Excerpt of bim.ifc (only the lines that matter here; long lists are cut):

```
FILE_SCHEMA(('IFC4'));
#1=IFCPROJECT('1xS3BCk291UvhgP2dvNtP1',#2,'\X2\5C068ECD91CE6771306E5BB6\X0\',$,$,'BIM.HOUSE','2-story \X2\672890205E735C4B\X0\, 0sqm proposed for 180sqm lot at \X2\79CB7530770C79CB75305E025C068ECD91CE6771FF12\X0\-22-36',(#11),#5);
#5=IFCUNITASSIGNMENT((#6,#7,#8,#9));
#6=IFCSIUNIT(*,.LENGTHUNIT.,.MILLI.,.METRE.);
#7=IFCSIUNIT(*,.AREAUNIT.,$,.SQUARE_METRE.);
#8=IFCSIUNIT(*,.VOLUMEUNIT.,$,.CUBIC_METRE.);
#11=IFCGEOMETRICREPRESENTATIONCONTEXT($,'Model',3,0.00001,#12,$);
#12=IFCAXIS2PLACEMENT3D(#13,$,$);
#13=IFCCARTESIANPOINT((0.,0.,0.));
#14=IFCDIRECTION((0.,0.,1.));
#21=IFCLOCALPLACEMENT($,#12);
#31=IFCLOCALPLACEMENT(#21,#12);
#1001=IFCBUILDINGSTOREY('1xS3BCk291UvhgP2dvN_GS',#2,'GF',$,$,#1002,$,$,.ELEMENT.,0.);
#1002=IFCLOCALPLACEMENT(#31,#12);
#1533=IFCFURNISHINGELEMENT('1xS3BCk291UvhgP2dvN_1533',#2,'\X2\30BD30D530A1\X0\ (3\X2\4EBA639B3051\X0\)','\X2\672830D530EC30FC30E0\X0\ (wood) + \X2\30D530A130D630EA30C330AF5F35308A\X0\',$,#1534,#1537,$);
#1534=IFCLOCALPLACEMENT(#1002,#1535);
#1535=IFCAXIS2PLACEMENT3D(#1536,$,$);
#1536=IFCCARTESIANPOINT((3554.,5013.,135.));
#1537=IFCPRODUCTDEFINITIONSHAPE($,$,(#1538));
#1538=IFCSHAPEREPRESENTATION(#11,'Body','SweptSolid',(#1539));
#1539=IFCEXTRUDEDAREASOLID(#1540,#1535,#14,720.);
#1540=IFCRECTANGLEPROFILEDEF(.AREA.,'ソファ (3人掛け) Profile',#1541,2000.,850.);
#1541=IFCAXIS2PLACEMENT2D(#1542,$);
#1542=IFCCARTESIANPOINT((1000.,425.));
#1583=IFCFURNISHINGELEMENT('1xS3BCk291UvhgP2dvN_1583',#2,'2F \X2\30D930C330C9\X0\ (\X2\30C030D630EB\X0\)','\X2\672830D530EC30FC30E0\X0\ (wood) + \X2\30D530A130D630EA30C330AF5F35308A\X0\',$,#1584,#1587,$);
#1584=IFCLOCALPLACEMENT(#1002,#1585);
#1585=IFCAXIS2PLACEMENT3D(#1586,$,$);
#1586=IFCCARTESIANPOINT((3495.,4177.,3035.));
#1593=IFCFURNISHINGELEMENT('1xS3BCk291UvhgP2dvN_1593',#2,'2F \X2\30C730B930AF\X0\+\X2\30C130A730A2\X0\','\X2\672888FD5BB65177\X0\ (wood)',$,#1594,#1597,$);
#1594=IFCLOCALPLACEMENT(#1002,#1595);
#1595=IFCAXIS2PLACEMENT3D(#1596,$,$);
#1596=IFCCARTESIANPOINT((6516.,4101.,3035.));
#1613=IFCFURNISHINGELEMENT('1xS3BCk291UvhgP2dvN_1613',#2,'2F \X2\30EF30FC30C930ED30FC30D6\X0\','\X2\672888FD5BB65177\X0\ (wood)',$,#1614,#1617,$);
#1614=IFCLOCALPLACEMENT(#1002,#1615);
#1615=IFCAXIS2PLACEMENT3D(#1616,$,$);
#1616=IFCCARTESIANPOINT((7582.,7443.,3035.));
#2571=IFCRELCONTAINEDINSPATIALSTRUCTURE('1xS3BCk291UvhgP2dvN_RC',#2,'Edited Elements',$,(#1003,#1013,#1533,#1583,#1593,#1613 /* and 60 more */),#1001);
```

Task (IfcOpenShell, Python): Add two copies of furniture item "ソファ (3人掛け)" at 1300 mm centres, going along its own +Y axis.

```python
import ifcopenshell
import ifcopenshell.api.geometry
import ifcopenshell.api.root
import ifcopenshell.util.element
import ifcopenshell.util.placement

model = ifcopenshell.open("bim.ifc")


def reuse_history(source, copy):
    """copy_class also copies each property set's owner history, people and application; keep the originals."""
    for rel in copy.IsDefinedBy:
        if rel.is_a("IfcRelDefinesByProperties") and (history := rel.RelatingPropertyDefinition.OwnerHistory):
            rel.RelatingPropertyDefinition.OwnerHistory = source.OwnerHistory
            ifcopenshell.util.element.remove_deep2(model, history)


source = model.by_id(1533)
base = ifcopenshell.util.placement.get_local_placement(source.ObjectPlacement)
step = base[:3, 1] * 1300.0

for i in range(1, 3):
    copy = ifcopenshell.api.root.copy_class(model, product=source)
    copy.Representation = ifcopenshell.util.element.copy_deep(
        model, source.Representation, exclude=["IfcGeometricRepresentationContext", "IfcRepresentationMap"]
    )
    reuse_history(source, copy)
    matrix = base.copy()
    matrix[:3, 3] += i * step
    print("added at", matrix[:3, 3].round(3) + 0.0)
    ifcopenshell.api.geometry.edit_object_placement(model, product=copy, matrix=matrix, is_si=False)

model.write("bim_v2.ifc")
```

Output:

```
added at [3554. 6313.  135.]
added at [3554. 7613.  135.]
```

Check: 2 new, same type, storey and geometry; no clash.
